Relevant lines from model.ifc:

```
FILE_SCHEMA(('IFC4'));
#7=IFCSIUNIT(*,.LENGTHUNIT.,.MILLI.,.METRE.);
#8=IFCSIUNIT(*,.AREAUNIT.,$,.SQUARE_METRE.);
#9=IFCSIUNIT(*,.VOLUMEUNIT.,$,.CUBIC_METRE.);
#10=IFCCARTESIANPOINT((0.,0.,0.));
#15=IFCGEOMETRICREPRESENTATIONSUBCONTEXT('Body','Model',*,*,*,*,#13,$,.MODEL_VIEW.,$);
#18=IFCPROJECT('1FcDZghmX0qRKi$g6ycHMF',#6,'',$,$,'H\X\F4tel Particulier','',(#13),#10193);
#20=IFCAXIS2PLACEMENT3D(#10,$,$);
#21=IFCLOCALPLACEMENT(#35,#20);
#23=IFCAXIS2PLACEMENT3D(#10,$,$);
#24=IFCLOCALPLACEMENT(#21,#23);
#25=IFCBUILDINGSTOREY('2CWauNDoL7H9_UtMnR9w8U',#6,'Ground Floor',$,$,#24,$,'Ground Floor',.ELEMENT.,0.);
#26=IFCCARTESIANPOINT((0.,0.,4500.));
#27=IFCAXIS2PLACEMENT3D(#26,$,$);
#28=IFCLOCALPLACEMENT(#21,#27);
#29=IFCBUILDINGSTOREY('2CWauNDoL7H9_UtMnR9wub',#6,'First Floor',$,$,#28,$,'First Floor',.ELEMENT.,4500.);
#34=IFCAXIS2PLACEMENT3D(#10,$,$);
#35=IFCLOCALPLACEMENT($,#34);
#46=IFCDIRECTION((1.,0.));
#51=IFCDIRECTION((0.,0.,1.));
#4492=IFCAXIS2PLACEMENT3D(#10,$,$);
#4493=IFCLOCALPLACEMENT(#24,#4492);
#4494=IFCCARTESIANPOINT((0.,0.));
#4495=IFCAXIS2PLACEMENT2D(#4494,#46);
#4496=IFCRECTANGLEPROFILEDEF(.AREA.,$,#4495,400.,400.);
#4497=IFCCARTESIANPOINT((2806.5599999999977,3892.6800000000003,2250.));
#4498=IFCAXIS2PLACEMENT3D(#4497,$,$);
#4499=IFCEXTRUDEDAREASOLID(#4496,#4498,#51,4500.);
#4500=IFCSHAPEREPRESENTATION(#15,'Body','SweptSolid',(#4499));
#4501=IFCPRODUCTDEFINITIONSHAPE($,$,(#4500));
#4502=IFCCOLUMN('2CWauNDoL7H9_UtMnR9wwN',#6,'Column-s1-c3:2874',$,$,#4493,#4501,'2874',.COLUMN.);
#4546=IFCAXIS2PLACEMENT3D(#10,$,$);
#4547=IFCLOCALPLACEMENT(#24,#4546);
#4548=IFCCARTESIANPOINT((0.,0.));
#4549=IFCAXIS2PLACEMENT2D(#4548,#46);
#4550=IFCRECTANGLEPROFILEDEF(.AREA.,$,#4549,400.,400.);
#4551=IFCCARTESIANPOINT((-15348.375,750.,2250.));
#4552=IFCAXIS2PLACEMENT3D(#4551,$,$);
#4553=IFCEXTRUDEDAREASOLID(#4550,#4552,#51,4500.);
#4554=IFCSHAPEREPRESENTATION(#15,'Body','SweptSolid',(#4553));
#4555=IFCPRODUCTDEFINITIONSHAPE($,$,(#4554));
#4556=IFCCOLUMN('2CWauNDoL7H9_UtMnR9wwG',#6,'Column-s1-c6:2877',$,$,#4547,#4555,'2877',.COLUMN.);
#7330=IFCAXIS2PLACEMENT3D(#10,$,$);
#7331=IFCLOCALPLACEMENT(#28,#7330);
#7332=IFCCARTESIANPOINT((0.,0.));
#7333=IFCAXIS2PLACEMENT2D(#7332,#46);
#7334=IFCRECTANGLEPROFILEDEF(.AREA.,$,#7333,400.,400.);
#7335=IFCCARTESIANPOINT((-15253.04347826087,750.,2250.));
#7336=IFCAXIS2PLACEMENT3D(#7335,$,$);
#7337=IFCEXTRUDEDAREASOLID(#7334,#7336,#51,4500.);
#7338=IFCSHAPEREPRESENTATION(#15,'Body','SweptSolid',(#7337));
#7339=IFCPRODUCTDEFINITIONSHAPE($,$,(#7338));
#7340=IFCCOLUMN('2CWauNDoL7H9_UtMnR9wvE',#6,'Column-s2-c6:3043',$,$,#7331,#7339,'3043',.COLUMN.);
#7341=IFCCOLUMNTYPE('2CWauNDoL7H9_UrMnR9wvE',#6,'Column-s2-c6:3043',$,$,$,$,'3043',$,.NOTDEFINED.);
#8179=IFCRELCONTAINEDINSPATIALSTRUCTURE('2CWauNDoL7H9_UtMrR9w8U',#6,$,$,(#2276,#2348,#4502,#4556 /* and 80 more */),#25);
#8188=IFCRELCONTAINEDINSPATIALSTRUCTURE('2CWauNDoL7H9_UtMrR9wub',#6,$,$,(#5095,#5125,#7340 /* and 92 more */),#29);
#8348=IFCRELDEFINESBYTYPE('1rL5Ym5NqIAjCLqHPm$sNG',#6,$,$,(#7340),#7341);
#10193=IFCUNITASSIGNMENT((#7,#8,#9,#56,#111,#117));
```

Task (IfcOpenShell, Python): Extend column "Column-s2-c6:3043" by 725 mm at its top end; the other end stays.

```python
import ifcopenshell
import ifcopenshell.util.representation
import ifcopenshell.util.unit

model = ifcopenshell.open("model.ifc")
unit_scale = ifcopenshell.util.unit.calculate_unit_scale(model)

member = model.by_guid("2CWauNDoL7H9_UtMnR9wvE")
change = 0.725 / unit_scale

# The extrusion runs towards the end named, so only its depth changes.
body = ifcopenshell.util.representation.get_representation(member, "Model", "Body")
solid = body.Items[0]
old_length = solid.Depth
solid.Depth += change

print(f"length {old_length:g} -> {solid.Depth:g}")

model.write("model_v2.ifc")
```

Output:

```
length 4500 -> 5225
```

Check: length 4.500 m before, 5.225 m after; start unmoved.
